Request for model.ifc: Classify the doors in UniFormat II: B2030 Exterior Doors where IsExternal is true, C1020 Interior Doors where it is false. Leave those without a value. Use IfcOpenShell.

First a look at what the model holds.

```python
import ifcopenshell
import ifcopenshell.util.element

model = ifcopenshell.open("model.ifc")
print(model.schema)
print("classifications:", [c.Name for c in model.by_type("IfcClassification")])
values = [ifcopenshell.util.element.get_pset(e, "Pset_DoorCommon", "IsExternal") for e in model.by_type("IfcDoor")]
for value in (True, False, None):
    print("IsExternal", value, values.count(value))
```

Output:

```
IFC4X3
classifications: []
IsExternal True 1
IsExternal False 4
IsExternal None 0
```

```python
import ifcopenshell
import ifcopenshell.api.classification
import ifcopenshell.util.element

model = ifcopenshell.open("model.ifc")

system = ifcopenshell.api.classification.add_classification(model, classification="UniFormat II")

doors = model.by_type("IfcDoor")
external = {e: ifcopenshell.util.element.get_pset(e, "Pset_DoorCommon", "IsExternal") for e in doors}
for flag, code, name in ((True, "B2030", "Exterior Doors"), (False, "C1020", "Interior Doors")):
    products = [e for e in doors if external[e] is flag]
    ifcopenshell.api.classification.add_reference(
        model, products=products, classification=system, identification=code, name=name
    )
    print(code, len(products))

model.write("model-out.ifc")
```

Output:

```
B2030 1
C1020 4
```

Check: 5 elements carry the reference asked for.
